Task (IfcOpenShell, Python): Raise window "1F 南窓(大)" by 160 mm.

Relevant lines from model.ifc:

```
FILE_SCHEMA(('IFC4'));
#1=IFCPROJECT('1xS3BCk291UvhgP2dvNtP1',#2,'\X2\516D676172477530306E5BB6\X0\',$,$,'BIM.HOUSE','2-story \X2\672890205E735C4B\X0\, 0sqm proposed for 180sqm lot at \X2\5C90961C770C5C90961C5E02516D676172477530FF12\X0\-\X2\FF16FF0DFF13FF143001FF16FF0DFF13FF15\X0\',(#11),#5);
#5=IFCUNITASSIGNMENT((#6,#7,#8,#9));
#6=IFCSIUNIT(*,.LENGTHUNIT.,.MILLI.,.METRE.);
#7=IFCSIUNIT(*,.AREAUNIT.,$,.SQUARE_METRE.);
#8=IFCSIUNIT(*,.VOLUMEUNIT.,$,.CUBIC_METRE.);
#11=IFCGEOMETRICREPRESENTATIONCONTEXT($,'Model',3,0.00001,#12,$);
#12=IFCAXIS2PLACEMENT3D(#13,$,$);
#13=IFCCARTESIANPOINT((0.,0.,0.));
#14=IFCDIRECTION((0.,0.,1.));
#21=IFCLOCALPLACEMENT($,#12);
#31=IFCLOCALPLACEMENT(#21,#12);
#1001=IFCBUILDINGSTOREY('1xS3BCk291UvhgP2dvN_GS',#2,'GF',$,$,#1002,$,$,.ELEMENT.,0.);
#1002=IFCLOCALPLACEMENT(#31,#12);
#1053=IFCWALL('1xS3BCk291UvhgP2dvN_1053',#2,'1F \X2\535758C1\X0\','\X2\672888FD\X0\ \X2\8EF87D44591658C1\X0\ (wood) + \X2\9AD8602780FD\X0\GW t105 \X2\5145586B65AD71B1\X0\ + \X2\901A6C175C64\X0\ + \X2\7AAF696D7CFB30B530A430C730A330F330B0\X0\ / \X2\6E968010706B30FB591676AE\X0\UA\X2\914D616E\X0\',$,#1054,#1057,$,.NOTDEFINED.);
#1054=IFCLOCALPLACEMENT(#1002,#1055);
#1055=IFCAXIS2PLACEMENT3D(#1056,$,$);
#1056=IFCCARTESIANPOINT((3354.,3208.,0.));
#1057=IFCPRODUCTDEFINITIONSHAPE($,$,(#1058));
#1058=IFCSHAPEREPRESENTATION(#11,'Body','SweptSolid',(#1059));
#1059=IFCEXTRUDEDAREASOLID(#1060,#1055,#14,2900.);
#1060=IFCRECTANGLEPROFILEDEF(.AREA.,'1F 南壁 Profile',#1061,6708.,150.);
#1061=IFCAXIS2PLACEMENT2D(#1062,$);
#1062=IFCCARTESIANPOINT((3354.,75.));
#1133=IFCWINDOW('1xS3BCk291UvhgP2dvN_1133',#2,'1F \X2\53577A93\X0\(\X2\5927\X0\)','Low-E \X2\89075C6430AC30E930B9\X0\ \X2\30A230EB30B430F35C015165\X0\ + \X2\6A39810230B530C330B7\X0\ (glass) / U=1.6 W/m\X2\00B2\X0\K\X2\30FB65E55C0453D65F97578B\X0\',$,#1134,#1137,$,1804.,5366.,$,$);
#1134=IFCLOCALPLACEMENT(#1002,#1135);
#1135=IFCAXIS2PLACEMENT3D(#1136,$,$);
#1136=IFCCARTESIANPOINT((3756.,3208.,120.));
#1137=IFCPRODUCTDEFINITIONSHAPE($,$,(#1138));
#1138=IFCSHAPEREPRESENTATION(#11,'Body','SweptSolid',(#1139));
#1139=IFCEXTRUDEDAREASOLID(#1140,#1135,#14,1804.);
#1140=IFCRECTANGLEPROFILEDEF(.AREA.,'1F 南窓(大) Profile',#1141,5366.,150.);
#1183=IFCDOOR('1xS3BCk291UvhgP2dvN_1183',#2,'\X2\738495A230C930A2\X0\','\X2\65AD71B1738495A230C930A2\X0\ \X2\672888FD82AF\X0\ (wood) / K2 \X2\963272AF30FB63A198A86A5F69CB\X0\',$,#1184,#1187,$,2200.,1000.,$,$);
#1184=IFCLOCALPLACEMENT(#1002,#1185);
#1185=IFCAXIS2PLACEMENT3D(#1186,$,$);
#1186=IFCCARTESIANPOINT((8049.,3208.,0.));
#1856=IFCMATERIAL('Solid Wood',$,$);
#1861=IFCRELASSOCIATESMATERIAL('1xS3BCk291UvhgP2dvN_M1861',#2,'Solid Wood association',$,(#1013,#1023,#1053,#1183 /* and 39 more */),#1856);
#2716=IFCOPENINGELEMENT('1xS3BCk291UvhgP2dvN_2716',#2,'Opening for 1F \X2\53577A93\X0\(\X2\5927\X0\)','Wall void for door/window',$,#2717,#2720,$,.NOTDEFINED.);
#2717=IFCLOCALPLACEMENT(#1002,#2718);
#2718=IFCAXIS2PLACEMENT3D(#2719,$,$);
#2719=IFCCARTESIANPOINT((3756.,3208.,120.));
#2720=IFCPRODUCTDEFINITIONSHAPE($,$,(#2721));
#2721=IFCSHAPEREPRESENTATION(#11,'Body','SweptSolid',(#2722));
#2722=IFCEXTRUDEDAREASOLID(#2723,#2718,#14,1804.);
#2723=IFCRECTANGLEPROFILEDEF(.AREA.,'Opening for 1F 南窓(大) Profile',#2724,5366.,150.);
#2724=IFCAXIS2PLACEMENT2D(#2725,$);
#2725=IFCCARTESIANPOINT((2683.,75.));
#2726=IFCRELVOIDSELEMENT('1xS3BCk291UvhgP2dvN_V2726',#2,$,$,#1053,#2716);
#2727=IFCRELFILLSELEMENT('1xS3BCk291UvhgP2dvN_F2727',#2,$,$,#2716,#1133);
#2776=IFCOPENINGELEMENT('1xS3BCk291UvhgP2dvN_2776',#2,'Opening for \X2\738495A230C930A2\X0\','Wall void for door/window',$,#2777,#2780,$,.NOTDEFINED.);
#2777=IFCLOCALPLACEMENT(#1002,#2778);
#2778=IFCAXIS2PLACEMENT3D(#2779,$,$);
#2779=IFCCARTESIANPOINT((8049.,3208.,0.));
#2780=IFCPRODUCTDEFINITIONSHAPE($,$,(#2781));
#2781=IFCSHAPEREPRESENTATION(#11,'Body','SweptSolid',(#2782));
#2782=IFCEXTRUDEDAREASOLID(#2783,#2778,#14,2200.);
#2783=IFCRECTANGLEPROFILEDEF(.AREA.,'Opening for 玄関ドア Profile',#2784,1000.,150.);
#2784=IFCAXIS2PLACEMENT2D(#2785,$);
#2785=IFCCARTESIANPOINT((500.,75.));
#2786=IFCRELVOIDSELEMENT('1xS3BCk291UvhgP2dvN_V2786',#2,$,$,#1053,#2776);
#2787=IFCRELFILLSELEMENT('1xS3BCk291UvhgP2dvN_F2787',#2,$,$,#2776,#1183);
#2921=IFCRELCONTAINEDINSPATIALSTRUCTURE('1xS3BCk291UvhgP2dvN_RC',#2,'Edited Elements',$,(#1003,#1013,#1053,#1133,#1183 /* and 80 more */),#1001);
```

```python
import numpy as np
import ifcopenshell
import ifcopenshell.api.geometry
import ifcopenshell.util.placement
import ifcopenshell.util.unit

model = ifcopenshell.open("model.ifc")
unit_scale = ifcopenshell.util.unit.calculate_unit_scale(model)

window = model.by_id(1133)
opening = window.FillsVoids[0].RelatingOpeningElement
dz = 0.16 / unit_scale

shift = np.array([0.0, 0.0, dz])
# The window is not placed relative to its opening, so move both.
for product in (opening, window):
    matrix = ifcopenshell.util.placement.get_local_placement(product.ObjectPlacement)
    matrix[:3, 3] += shift
    ifcopenshell.api.geometry.edit_object_placement(model, product=product, matrix=matrix, is_si=False)

print(f"moved by {dz * unit_scale:+.3f} m")

model.write("model_updated.ifc")
```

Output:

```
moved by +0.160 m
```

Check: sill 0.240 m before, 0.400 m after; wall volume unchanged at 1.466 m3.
